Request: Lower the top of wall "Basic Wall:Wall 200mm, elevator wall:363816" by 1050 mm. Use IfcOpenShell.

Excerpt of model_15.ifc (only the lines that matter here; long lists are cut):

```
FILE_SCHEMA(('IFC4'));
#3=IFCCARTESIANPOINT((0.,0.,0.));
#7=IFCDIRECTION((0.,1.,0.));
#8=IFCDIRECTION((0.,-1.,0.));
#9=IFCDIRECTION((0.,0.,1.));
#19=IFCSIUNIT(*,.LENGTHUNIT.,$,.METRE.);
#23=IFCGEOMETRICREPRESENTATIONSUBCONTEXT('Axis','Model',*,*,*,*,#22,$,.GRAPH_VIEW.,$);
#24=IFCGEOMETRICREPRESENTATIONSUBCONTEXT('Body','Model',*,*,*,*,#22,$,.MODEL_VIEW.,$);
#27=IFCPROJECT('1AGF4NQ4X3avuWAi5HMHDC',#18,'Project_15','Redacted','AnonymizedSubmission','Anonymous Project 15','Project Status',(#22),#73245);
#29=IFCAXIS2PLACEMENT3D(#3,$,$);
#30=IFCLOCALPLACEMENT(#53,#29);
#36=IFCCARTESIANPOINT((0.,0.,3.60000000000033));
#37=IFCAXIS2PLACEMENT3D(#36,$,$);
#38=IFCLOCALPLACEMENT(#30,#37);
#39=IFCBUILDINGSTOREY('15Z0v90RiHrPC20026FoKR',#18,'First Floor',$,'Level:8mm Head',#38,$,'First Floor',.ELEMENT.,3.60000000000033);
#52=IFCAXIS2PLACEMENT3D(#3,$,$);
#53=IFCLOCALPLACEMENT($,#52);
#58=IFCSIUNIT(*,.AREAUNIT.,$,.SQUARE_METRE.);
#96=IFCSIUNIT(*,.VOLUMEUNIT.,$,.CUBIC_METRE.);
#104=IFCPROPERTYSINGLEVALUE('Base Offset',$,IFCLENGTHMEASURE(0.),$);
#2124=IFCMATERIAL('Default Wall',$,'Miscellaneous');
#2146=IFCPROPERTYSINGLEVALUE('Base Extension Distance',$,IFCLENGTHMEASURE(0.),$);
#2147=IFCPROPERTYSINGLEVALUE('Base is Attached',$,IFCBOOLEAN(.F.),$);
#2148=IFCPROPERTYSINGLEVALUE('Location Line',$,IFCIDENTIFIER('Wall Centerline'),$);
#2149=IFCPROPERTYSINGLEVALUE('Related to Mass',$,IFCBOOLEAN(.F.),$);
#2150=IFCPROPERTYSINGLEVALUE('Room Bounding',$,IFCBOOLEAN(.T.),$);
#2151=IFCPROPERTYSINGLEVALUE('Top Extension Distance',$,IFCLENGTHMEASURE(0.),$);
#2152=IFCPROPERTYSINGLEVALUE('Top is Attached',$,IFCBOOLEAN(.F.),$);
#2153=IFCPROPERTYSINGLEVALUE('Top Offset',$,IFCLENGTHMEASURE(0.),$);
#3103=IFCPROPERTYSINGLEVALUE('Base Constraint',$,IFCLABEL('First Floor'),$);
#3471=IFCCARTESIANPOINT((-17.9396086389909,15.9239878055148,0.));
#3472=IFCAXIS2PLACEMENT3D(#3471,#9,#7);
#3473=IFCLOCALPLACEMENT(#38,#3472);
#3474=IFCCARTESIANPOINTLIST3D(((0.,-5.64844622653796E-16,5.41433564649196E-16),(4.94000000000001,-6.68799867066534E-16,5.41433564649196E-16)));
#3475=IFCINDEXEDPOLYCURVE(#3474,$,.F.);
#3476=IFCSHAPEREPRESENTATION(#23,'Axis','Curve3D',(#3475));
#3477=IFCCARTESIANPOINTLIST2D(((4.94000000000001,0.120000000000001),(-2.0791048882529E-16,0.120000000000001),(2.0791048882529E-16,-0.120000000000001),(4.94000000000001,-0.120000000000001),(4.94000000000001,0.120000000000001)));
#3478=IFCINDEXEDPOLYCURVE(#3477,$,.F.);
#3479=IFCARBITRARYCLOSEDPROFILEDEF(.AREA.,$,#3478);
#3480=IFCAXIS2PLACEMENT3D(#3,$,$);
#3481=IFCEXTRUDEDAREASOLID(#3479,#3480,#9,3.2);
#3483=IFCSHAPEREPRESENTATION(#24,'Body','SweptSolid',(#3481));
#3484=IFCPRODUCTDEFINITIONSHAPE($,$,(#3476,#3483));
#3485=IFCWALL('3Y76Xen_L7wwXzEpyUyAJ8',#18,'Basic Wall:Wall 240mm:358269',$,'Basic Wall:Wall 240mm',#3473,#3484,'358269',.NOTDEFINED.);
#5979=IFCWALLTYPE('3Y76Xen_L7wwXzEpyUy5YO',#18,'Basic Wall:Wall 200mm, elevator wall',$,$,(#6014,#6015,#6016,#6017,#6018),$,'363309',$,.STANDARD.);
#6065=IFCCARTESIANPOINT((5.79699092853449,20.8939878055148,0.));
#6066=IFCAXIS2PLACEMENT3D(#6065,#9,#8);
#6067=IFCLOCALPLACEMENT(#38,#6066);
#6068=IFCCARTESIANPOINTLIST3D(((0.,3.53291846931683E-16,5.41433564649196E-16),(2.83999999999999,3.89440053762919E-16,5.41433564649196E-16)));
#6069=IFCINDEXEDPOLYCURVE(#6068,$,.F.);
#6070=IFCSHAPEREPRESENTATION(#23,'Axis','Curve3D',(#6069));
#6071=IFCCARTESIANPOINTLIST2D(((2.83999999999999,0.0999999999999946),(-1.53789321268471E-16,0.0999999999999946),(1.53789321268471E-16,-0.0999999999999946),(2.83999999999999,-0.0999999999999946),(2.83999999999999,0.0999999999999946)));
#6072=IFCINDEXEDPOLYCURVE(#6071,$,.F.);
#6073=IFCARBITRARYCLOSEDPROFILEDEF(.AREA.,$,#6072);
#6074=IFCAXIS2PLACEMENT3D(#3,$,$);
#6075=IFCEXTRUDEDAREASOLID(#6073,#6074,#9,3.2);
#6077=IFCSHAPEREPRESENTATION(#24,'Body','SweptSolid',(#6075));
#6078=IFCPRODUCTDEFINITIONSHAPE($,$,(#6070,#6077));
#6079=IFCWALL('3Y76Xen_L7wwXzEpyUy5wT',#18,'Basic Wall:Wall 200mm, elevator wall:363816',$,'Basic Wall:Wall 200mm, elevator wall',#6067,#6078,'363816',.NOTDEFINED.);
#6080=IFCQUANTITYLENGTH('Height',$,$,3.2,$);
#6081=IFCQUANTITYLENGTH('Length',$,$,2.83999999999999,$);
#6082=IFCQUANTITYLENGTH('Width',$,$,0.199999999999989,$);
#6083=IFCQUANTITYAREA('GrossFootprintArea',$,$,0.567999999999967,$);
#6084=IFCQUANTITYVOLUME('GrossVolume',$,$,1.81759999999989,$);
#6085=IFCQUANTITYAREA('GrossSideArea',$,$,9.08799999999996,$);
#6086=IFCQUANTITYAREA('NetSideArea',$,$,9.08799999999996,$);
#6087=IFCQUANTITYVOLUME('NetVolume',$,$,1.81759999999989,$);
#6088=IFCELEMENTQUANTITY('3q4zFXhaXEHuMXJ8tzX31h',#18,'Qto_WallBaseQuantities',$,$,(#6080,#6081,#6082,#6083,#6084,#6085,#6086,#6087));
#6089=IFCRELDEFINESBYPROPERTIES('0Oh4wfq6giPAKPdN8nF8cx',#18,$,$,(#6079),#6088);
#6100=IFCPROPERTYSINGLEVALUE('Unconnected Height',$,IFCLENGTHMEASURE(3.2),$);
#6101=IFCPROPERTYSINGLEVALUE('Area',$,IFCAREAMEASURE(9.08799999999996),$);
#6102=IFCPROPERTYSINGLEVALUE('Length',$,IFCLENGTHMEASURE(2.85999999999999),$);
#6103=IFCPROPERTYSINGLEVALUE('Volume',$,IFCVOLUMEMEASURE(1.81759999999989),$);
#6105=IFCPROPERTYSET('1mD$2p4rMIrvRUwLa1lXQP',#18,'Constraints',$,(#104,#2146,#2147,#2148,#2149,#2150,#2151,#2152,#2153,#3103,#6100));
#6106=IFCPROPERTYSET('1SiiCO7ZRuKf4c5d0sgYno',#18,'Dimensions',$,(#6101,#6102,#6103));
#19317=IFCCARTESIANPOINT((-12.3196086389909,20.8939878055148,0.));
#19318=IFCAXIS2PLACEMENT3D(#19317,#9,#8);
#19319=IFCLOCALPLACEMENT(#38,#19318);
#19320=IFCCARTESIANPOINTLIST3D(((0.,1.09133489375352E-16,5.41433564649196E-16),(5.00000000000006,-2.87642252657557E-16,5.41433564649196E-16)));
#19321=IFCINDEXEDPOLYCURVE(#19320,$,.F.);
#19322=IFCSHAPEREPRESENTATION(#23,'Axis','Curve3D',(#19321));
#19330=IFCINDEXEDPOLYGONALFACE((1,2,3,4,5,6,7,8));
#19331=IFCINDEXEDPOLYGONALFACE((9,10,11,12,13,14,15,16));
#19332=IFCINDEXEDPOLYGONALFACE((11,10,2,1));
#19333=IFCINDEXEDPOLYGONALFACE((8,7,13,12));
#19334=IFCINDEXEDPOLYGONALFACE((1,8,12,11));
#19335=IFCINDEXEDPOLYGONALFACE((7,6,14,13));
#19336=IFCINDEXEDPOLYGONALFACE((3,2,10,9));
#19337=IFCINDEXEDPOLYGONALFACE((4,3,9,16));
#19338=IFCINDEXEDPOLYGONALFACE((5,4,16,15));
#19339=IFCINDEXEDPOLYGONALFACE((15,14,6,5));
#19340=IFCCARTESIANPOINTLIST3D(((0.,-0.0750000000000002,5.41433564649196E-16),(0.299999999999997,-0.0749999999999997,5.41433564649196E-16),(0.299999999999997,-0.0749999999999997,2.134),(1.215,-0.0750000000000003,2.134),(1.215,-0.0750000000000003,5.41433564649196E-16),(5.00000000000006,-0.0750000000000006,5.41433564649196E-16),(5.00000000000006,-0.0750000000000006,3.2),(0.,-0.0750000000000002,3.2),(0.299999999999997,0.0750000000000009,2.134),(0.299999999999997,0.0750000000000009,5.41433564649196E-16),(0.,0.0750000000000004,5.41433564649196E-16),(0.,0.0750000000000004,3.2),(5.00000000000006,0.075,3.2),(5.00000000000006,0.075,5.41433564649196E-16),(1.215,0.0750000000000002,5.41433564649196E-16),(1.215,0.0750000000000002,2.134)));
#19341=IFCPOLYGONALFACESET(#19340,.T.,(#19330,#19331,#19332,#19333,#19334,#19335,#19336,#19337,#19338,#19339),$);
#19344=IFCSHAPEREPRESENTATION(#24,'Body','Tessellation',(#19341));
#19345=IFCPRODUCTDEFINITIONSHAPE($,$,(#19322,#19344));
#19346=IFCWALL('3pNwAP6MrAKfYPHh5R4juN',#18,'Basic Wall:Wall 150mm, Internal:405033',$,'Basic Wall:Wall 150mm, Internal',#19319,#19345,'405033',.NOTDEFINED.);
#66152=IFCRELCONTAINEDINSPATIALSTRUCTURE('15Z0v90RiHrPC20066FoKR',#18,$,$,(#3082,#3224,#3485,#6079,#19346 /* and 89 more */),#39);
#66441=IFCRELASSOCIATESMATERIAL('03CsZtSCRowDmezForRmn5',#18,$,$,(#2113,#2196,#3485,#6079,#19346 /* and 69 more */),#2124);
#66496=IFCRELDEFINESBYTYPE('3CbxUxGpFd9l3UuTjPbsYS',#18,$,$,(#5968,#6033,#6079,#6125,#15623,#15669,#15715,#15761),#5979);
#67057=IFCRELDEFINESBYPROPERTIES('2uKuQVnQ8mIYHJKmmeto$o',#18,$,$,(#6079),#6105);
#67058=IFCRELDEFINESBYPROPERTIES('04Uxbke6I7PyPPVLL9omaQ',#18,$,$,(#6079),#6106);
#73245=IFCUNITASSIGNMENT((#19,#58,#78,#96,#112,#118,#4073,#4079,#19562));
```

```python
import ifcopenshell
import ifcopenshell.api.pset
import ifcopenshell.geom
import ifcopenshell.util.element
import ifcopenshell.util.representation
import ifcopenshell.util.shape
import ifcopenshell.util.unit

model = ifcopenshell.open("model_15.ifc")
unit_scale = ifcopenshell.util.unit.calculate_unit_scale(model)
area_scale = ifcopenshell.util.unit.calculate_unit_scale(model, "AREAUNIT")
volume_scale = ifcopenshell.util.unit.calculate_unit_scale(model, "VOLUMEUNIT")
settings = ifcopenshell.geom.settings()


def volume(element):
    """Net volume in cubic metres, openings subtracted."""
    shape = ifcopenshell.geom.create_shape(settings, element)
    return ifcopenshell.util.shape.get_volume(shape.geometry)


wall = model.by_guid("3Y76Xen_L7wwXzEpyUy5wT")
before = volume(wall)

body = ifcopenshell.util.representation.get_representation(wall, "Model", "Body")
solid = body.Items[0]
old_height = solid.Depth
solid.Depth -= 1.05 / unit_scale
after = volume(wall)
thickness = 0.2  # wall thickness in metres

# Update the stored height, areas and volumes.
qto = model.by_id(ifcopenshell.util.element.get_pset(wall, "Qto_WallBaseQuantities", should_inherit=False)["id"])
ifcopenshell.api.pset.edit_qto(model, qto=qto, properties={
    "Height": solid.Depth,
    "GrossVolume": ifcopenshell.util.element.get_pset(wall, "Qto_WallBaseQuantities", "GrossVolume") * solid.Depth / old_height,
    "GrossSideArea": ifcopenshell.util.element.get_pset(wall, "Qto_WallBaseQuantities", "GrossSideArea") * solid.Depth / old_height,
    "NetSideArea": after / thickness / area_scale,
    "NetVolume": after / volume_scale,
})
pset = model.by_id(ifcopenshell.util.element.get_pset(wall, "Constraints", should_inherit=False)["id"])
ifcopenshell.api.pset.edit_pset(model, pset=pset, properties={
    "Unconnected Height": model.create_entity("IfcLengthMeasure", solid.Depth),
})
pset = model.by_id(ifcopenshell.util.element.get_pset(wall, "Dimensions", should_inherit=False)["id"])
ifcopenshell.api.pset.edit_pset(model, pset=pset, properties={
    "Area": model.create_entity("IfcAreaMeasure", after / thickness / area_scale),
    "Volume": model.create_entity("IfcVolumeMeasure", after / volume_scale),
})

print(f"height {old_height:g} -> {solid.Depth:g}, volume {before:.3f} -> {after:.3f} m3")

model.write("model_15_rev.ifc")
```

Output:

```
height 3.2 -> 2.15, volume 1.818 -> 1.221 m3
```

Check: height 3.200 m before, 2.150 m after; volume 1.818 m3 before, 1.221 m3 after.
